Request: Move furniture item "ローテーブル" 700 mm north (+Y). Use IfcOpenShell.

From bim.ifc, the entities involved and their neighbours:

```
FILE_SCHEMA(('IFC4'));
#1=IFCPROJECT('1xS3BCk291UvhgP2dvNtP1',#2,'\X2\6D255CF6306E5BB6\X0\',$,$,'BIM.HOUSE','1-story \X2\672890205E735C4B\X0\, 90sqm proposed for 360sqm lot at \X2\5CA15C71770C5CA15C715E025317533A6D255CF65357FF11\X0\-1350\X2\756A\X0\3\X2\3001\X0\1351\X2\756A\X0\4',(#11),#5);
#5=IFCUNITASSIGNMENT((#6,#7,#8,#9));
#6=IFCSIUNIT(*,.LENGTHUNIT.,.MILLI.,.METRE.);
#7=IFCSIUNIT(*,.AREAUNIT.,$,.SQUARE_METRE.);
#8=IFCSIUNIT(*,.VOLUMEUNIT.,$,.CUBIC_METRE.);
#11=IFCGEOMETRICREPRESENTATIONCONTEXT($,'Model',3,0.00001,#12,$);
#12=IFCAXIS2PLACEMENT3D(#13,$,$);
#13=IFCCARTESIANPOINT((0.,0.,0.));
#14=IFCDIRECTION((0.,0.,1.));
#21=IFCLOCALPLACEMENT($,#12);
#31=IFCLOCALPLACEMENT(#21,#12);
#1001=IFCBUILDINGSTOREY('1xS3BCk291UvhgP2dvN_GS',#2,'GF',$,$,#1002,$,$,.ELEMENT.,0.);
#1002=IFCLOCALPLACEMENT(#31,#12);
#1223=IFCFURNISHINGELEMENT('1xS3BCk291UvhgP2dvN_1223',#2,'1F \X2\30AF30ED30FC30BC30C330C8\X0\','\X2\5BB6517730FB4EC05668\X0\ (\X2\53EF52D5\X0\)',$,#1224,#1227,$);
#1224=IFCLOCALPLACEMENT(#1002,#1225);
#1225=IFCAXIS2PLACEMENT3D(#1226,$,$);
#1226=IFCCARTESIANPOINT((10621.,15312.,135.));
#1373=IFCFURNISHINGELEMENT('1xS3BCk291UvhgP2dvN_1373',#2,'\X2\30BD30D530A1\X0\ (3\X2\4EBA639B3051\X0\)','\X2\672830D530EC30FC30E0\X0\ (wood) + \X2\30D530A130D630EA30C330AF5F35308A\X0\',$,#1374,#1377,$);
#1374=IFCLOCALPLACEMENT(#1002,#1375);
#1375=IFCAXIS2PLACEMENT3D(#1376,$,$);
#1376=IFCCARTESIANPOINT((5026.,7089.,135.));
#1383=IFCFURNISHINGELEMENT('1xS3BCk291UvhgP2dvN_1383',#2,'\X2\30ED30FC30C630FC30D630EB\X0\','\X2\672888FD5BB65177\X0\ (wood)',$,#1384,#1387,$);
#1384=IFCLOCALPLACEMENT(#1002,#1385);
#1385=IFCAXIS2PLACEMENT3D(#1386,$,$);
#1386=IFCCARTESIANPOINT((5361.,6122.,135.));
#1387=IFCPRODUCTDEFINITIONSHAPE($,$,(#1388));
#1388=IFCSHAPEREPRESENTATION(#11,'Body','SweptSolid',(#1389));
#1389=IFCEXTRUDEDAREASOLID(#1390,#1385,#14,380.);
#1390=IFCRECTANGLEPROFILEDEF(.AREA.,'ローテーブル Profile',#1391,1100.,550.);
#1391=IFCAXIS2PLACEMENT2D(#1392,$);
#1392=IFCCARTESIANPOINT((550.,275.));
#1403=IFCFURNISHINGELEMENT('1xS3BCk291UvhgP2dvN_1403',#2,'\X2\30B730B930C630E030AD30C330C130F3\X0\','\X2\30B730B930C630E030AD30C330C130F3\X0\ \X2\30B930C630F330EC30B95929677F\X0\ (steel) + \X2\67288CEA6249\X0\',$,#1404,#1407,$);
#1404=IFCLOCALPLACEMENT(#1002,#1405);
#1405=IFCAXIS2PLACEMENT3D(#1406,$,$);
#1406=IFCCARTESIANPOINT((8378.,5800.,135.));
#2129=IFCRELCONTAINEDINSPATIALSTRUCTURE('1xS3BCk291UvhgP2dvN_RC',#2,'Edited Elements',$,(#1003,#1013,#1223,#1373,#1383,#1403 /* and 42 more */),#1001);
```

```python
import ifcopenshell
import ifcopenshell.api.geometry
import ifcopenshell.util.placement
import ifcopenshell.util.unit

model = ifcopenshell.open("bim.ifc")
unit_scale = ifcopenshell.util.unit.calculate_unit_scale(model)

item = model.by_guid("1xS3BCk291UvhgP2dvN_1383")
matrix = ifcopenshell.util.placement.get_local_placement(item.ObjectPlacement)
matrix[1, 3] += 0.7 / unit_scale
ifcopenshell.api.geometry.edit_object_placement(model, product=item, matrix=matrix, is_si=False)

print(ifcopenshell.util.placement.get_local_placement(item.ObjectPlacement).round(3) + 0.0)

model.write("bim_edited.ifc")
```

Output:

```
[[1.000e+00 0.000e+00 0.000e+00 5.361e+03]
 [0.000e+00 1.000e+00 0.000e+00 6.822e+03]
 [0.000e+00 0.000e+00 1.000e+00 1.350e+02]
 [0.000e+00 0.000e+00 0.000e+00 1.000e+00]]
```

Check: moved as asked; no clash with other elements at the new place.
